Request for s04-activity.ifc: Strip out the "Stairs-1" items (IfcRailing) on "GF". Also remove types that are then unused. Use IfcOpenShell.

First a look at what the model holds.

```python
import ifcopenshell
import ifcopenshell.util.element

model = ifcopenshell.open("s04-activity.ifc")
print(model.schema)
storey = next(s for s in model.by_type("IfcBuildingStorey") if s.Name == "GF")
railings = [e for e in ifcopenshell.util.element.get_decomposition(storey) if e.is_a("IfcRailing")]
seen = {}
for e in railings:
    element_type = ifcopenshell.util.element.get_type(e)
    name = element_type.Name if element_type not in (None, e) else None
    seen[name] = seen.get(name, 0) + 1
for name, count in sorted(seen.items(), key=str):
    print(count, "x", name)
```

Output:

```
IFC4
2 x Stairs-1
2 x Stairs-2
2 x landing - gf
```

```python
import ifcopenshell
import ifcopenshell.api.root
import ifcopenshell.util.element

model = ifcopenshell.open("s04-activity.ifc")

storey = next(s for s in model.by_type("IfcBuildingStorey") if s.Name == "GF")
railings = [e for e in ifcopenshell.util.element.get_decomposition(storey) if e.is_a("IfcRailing")]
targets = [e for e in railings if (t := ifcopenshell.util.element.get_type(e)) not in (None, e) and t.Name == "Stairs-1"]
types = {ifcopenshell.util.element.get_type(e) for e in targets} - {None, *targets}

for e in targets:
    ifcopenshell.api.root.remove_product(model, product=e)
print(len(targets), "removed")

unused = [t for t in types if not ifcopenshell.util.element.get_types(t)]
for t in unused:
    ifcopenshell.api.root.remove_product(model, product=t)
print(len(unused), "unused types removed")

model.write("s04-activity_updated.ifc")
```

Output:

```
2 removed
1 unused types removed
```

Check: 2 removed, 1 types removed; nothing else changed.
